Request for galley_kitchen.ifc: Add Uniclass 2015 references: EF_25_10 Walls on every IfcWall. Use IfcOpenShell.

First a look at what the model holds.

```python
import ifcopenshell

model = ifcopenshell.open("galley_kitchen.ifc")
print(model.schema)
print("classifications:", [c.Name for c in model.by_type("IfcClassification")])
for ifc_class in ("IfcDoor", "IfcRoof", "IfcStair", "IfcWall", "IfcWindow"):
    print(ifc_class, len(model.by_type(ifc_class)))
```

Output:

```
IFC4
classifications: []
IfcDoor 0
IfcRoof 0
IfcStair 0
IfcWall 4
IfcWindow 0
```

```python
import ifcopenshell
import ifcopenshell.api.classification

model = ifcopenshell.open("galley_kitchen.ifc")

system = ifcopenshell.api.classification.add_classification(model, classification="Uniclass 2015")

codes = {
    "IfcWall": ("EF_25_10", "Walls"),
}
for ifc_class, (code, name) in codes.items():
    products = model.by_type(ifc_class)
    ifcopenshell.api.classification.add_reference(
        model, products=products, classification=system, identification=code, name=name
    )
    print(code, len(products))

model.write("galley_kitchen_updated.ifc")
```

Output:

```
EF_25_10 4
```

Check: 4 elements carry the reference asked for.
